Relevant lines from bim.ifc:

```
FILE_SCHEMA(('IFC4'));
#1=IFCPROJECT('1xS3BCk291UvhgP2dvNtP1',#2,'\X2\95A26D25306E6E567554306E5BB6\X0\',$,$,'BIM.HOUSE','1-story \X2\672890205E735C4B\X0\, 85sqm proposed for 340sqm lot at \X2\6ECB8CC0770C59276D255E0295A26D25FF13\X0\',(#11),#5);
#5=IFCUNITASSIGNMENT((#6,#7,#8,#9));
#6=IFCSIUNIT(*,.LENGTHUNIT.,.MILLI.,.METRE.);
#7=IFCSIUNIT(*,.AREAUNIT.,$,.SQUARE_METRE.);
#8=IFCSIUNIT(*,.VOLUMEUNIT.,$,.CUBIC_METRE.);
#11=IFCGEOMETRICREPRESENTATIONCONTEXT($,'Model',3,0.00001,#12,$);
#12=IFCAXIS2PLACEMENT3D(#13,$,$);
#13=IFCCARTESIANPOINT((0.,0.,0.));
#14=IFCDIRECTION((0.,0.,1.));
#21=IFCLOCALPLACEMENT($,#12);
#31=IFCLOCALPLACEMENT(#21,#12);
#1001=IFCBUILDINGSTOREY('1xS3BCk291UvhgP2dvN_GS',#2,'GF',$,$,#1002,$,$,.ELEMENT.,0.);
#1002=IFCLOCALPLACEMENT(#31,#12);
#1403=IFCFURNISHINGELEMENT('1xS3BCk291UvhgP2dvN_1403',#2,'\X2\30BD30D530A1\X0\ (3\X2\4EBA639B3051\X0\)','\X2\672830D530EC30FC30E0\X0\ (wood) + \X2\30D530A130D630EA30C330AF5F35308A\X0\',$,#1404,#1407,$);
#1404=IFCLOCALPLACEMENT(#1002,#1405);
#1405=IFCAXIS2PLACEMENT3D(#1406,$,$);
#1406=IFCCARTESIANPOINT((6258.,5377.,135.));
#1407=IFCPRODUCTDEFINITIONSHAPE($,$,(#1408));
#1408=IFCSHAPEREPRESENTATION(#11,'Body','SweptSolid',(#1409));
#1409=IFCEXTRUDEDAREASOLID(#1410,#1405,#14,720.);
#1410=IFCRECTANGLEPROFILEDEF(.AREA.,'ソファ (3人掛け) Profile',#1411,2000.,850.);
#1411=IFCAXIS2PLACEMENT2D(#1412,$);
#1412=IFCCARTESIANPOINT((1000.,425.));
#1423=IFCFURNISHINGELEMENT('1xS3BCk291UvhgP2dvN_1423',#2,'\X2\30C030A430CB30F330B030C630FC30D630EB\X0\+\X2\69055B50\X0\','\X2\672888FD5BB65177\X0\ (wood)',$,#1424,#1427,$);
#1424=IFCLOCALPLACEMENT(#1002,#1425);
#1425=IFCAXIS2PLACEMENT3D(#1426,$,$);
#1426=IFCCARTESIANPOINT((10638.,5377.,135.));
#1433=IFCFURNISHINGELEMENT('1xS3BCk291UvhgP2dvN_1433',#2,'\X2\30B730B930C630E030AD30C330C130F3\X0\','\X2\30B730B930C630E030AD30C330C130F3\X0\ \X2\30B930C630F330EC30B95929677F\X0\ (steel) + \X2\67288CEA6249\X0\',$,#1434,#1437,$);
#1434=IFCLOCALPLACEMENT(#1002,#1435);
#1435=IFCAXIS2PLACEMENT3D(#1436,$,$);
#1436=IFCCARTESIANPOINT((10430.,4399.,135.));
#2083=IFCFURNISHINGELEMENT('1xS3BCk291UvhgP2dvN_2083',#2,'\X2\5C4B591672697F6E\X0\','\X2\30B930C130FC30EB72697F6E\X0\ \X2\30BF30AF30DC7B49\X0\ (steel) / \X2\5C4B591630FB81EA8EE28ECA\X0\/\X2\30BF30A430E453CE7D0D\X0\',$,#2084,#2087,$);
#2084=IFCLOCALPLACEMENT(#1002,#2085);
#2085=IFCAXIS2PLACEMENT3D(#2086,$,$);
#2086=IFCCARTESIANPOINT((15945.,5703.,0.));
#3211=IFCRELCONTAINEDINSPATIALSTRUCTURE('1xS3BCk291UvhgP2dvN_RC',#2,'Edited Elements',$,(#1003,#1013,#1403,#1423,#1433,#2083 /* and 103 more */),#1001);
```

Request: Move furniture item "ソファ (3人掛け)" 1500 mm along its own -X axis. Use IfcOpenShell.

```python
import ifcopenshell
import ifcopenshell.api.geometry
import ifcopenshell.util.placement
import ifcopenshell.util.unit

model = ifcopenshell.open("bim.ifc")
unit_scale = ifcopenshell.util.unit.calculate_unit_scale(model)

item = model.by_id(1403)
matrix = ifcopenshell.util.placement.get_local_placement(item.ObjectPlacement)
matrix[:3, 3] -= matrix[:3, 0] * 1.5 / unit_scale
ifcopenshell.api.geometry.edit_object_placement(model, product=item, matrix=matrix, is_si=False)

print(ifcopenshell.util.placement.get_local_placement(item.ObjectPlacement).round(3) + 0.0)

model.write("bim_edited.ifc")
```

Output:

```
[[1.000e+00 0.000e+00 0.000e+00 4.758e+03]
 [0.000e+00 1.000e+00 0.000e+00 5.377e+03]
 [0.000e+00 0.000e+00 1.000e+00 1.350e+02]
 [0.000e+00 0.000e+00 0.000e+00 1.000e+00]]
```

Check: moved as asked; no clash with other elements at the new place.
